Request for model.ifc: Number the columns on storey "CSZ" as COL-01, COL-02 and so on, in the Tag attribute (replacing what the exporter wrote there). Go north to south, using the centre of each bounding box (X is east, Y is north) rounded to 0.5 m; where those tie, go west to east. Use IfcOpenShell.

First a look at what the model holds.

```python
import ifcopenshell
import ifcopenshell.util.element
import ifcopenshell.util.placement

model = ifcopenshell.open("model.ifc")
print(model.schema)
storey = next(s for s in model.by_type("IfcBuildingStorey") if s.Name == "CSZ")
columns = [e for e in ifcopenshell.util.element.get_decomposition(storey) if e.is_a("IfcColumn")]
for e in sorted(columns, key=lambda e: e.id()):
    origin = ifcopenshell.util.placement.get_local_placement(e.ObjectPlacement)[:3, 3]
    print(e.id(), e.Tag, e.Name, origin.round(2) + 0.0, sep=" | ")
```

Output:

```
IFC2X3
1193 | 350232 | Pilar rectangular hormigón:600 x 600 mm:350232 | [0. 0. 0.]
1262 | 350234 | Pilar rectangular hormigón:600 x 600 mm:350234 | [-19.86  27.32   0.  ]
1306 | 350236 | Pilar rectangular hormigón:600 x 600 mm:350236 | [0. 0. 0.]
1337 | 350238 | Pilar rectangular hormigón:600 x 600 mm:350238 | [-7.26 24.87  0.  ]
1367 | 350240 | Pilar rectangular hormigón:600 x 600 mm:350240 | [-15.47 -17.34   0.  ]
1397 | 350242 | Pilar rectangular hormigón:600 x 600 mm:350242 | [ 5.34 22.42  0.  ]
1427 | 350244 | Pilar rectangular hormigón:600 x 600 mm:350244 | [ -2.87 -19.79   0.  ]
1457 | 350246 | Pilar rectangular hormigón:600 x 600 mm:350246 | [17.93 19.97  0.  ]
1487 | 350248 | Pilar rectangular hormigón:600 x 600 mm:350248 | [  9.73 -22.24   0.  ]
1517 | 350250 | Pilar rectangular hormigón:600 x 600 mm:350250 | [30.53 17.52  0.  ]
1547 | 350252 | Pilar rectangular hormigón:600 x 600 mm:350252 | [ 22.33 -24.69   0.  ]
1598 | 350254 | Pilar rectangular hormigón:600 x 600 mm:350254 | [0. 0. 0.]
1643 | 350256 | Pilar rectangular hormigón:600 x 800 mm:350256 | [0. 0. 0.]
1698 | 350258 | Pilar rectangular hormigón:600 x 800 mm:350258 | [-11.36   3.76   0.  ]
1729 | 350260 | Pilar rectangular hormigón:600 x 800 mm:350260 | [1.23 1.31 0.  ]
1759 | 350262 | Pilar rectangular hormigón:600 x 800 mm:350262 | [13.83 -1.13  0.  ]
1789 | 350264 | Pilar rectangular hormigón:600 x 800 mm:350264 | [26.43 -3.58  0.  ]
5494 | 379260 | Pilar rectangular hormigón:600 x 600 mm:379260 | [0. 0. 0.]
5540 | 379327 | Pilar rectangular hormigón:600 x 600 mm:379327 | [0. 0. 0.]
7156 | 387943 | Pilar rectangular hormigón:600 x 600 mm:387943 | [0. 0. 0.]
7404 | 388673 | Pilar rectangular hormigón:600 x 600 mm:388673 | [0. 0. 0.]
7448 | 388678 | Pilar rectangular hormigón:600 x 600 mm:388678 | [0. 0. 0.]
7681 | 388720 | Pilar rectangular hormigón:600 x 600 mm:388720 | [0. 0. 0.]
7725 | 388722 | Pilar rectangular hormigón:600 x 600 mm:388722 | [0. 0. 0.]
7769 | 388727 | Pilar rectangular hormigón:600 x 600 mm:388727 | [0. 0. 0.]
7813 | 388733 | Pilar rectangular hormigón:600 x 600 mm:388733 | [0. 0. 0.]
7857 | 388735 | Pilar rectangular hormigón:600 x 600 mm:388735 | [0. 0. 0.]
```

```python
import ifcopenshell
import ifcopenshell.geom
import ifcopenshell.util.element
import ifcopenshell.util.shape

model = ifcopenshell.open("model.ifc")
settings = ifcopenshell.geom.settings()
settings.set("use-world-coords", True)


def centre(element):
    shape = ifcopenshell.geom.create_shape(settings, element)
    return ifcopenshell.util.shape.get_bbox_centroid(shape.geometry)


storey = next(s for s in model.by_type("IfcBuildingStorey") if s.Name == "CSZ")
columns = [e for e in ifcopenshell.util.element.get_decomposition(storey) if e.is_a("IfcColumn")]

# Insertion points can sit at a corner or the storey origin, so sort by the geometry (in metres).
centres = {e: centre(e) for e in columns}
columns.sort(key=lambda e: (-round(centres[e][1] / 0.5), centres[e][0]))

for i, e in enumerate(columns, start=1):
    number = f"COL-{i:02d}"
    e.Tag = number
    print(e.id(), number)

model.write("model_updated.ifc")
```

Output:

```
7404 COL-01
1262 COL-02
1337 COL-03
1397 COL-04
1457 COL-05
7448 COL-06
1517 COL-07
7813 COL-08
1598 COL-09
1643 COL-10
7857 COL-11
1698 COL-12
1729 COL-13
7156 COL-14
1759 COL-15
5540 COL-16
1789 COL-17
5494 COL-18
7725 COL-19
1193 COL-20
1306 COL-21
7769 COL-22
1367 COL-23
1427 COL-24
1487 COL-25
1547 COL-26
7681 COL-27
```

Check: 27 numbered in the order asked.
